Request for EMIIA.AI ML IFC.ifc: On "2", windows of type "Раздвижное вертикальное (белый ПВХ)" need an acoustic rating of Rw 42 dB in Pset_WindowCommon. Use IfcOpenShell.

First a look at what the model holds.

```python
import ifcopenshell
import ifcopenshell.util.element

model = ifcopenshell.open("EMIIA.AI ML IFC.ifc")
print(model.schema)
storey = next(s for s in model.by_type("IfcBuildingStorey") if s.Name == "2")
windows = [e for e in ifcopenshell.util.element.get_decomposition(storey) if e.is_a("IfcWindow")]
seen = {}
for e in windows:
    element_type = ifcopenshell.util.element.get_type(e)
    key = (element_type.Name if element_type != e and element_type else None, ifcopenshell.util.element.get_pset(e, "Pset_WindowCommon", "AcousticRating"))
    seen[key] = seen.get(key, 0) + 1
for (name, value), count in sorted(seen.items(), key=str):
    print(count, "x", name, "|", value)
```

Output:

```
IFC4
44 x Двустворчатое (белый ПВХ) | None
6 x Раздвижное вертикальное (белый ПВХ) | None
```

```python
import ifcopenshell
import ifcopenshell.api.pset
import ifcopenshell.util.element

model = ifcopenshell.open("EMIIA.AI ML IFC.ifc")

storey = next(s for s in model.by_type("IfcBuildingStorey") if s.Name == "2")
windows = [e for e in ifcopenshell.util.element.get_decomposition(storey) if e.is_a("IfcWindow")]

count = 0
for e in windows:
    element_type = ifcopenshell.util.element.get_type(e)
    if element_type in (None, e) or element_type.Name != "Раздвижное вертикальное (белый ПВХ)":
        continue
    # add_pset returns the element's existing set when there is one.
    pset = ifcopenshell.api.pset.add_pset(model, product=e, name="Pset_WindowCommon")
    ifcopenshell.api.pset.edit_pset(model, pset=pset, properties={"AcousticRating": "Rw 42 dB"})
    count += 1

print(count, "windows updated")

model.write("EMIIA.AI ML IFC-out.ifc")
```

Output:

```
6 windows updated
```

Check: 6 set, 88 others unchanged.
